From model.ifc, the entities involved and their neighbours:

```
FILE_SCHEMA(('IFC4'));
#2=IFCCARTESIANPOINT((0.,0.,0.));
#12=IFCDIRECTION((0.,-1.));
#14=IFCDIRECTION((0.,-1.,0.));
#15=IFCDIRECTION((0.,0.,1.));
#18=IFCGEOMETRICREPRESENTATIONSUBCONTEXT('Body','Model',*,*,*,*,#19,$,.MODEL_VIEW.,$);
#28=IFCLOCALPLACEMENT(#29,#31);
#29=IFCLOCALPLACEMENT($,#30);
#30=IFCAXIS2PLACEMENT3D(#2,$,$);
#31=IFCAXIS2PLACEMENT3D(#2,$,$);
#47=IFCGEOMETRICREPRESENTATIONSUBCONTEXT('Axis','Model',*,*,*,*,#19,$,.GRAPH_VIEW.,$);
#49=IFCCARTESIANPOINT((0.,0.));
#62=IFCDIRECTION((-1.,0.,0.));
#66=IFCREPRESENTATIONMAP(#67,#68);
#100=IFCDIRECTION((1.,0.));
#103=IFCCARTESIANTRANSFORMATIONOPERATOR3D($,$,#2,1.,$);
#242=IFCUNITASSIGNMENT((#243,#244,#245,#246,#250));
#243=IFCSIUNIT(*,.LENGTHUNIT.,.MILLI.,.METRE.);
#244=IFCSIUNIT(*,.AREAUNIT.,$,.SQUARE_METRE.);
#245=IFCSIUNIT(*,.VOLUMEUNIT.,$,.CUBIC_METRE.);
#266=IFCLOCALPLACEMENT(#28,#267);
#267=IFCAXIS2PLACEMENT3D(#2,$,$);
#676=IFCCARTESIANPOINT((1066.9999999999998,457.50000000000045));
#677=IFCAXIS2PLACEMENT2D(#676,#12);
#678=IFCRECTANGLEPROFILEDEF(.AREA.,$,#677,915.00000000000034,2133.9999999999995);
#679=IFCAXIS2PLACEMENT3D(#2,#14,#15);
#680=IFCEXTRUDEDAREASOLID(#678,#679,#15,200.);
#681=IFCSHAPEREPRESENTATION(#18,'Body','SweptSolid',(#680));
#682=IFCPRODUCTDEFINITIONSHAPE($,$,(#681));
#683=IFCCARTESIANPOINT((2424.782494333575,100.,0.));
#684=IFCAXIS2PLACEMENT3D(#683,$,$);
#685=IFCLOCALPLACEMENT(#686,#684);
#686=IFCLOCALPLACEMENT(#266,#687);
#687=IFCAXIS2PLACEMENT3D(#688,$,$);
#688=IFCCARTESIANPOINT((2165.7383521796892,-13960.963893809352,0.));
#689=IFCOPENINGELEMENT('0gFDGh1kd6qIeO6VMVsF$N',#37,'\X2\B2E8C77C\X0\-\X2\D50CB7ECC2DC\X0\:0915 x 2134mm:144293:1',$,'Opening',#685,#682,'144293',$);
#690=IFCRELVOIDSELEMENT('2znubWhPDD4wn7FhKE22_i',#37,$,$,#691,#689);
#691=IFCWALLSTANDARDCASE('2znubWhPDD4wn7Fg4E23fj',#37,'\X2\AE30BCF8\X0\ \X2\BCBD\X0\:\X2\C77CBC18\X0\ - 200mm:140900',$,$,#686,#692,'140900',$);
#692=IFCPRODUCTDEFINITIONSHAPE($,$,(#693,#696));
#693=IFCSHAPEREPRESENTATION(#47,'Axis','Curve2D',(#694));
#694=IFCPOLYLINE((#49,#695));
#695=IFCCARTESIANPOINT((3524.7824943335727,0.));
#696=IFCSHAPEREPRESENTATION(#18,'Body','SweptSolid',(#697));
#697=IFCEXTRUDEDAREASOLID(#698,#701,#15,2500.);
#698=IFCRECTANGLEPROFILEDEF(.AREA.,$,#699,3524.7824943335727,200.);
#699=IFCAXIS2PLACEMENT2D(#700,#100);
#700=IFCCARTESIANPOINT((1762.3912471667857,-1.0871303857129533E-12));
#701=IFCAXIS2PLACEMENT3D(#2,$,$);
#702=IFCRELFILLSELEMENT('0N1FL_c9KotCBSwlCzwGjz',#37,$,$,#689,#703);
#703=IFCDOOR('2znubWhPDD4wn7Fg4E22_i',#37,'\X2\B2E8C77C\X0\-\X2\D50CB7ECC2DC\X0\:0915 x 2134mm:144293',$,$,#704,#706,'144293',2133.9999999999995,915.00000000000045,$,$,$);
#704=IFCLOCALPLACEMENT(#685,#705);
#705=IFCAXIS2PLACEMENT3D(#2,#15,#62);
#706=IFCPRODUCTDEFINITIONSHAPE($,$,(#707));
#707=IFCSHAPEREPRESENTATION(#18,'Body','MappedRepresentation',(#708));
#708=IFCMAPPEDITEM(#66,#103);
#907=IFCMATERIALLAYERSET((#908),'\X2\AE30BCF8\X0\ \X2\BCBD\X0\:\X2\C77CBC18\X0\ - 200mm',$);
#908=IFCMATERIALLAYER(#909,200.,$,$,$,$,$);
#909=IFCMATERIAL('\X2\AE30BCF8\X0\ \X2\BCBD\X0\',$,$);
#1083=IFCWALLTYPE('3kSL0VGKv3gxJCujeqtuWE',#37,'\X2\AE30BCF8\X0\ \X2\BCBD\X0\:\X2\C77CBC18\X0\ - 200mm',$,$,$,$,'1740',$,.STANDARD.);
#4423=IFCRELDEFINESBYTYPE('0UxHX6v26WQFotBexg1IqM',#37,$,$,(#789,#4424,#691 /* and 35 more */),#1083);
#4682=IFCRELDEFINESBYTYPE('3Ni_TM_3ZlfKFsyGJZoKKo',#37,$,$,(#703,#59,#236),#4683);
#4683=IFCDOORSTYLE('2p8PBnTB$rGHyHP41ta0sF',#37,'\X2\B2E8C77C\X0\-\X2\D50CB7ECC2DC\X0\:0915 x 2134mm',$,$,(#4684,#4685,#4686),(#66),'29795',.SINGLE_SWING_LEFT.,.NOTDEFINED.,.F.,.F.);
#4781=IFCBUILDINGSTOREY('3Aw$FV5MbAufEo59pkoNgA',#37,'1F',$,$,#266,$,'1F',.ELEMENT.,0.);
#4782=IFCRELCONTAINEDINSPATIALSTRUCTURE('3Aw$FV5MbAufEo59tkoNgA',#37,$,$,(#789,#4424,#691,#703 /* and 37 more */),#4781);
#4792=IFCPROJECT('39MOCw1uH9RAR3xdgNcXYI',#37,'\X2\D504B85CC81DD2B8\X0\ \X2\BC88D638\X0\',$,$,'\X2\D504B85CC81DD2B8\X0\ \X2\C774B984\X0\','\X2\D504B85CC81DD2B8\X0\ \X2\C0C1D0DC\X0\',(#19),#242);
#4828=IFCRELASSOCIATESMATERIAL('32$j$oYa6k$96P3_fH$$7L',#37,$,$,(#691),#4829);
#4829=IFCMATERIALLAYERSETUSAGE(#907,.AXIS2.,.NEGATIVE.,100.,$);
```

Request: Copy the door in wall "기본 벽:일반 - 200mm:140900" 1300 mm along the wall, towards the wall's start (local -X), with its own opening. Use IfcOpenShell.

```python
import ifcopenshell
import ifcopenshell.api.feature
import ifcopenshell.api.geometry
import ifcopenshell.api.root
import ifcopenshell.geom
import ifcopenshell.util.element
import ifcopenshell.util.placement
import ifcopenshell.util.shape
import ifcopenshell.util.unit

model = ifcopenshell.open("model.ifc")
unit_scale = ifcopenshell.util.unit.calculate_unit_scale(model)
settings = ifcopenshell.geom.settings()


def volume(element):
    """Net volume in cubic metres, openings subtracted."""
    shape = ifcopenshell.geom.create_shape(settings, element)
    return ifcopenshell.util.shape.get_volume(shape.geometry)


def reuse_history(source, copy):
    """copy_class also copies each property set's owner history, people and application; keep the originals."""
    for rel in copy.IsDefinedBy:
        if rel.is_a("IfcRelDefinesByProperties") and (history := rel.RelatingPropertyDefinition.OwnerHistory):
            rel.RelatingPropertyDefinition.OwnerHistory = source.OwnerHistory
            ifcopenshell.util.element.remove_deep2(model, history)


door = model.by_id(703)
opening = door.FillsVoids[0].RelatingOpeningElement
wall = opening.VoidsElements[0].RelatingBuildingElement
before = volume(wall)
shift = ifcopenshell.util.placement.get_local_placement(wall.ObjectPlacement)[:3, 0] * -1.3 / unit_scale

# copy_class copies the void relationship, type, container and properties, but no geometry.
new_opening = ifcopenshell.api.root.copy_class(model, product=opening)
new_opening.Representation = ifcopenshell.util.element.copy_deep(
    model, opening.Representation, exclude=["IfcGeometricRepresentationContext", "IfcRepresentationMap"]
)
new_opening.Name = "단일-플러시:0915 x 2134mm"
new_opening.Tag = None
new_door = ifcopenshell.api.root.copy_class(model, product=door)
new_door.Representation = ifcopenshell.util.element.copy_deep(
    model, door.Representation, exclude=["IfcGeometricRepresentationContext", "IfcRepresentationMap"]
)
new_door.Name = "단일-플러시:0915 x 2134mm"
new_door.Tag = None
reuse_history(door, new_door)
ifcopenshell.api.feature.add_filling(model, opening=new_opening, element=new_door)

for old, new in ((opening, new_opening), (door, new_door)):
    matrix = ifcopenshell.util.placement.get_local_placement(old.ObjectPlacement)
    matrix[:3, 3] += shift
    ifcopenshell.api.geometry.edit_object_placement(model, product=new, matrix=matrix, is_si=False)

after = volume(wall)

print(f"wall volume {before:.3f} -> {after:.3f} m3")

model.write("model_v2.ifc")
```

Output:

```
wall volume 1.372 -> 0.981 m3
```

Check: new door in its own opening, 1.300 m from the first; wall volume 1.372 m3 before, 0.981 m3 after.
